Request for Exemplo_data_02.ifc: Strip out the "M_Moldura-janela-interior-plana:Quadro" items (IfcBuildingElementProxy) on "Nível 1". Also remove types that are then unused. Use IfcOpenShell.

First a look at what the model holds.

```python
import ifcopenshell
import ifcopenshell.util.element

model = ifcopenshell.open("Exemplo_data_02.ifc")
print(model.schema)
storey = next(s for s in model.by_type("IfcBuildingStorey") if s.Name == "Nível 1")
proxies = [e for e in ifcopenshell.util.element.get_decomposition(storey) if e.is_a("IfcBuildingElementProxy")]
seen = {}
for e in proxies:
    element_type = ifcopenshell.util.element.get_type(e)
    name = element_type.Name if element_type not in (None, e) else None
    seen[name] = seen.get(name, 0) + 1
for name, count in sorted(seen.items(), key=str):
    print(count, "x", name)
```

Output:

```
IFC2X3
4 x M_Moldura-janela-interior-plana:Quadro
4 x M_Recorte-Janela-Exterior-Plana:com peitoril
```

```python
import ifcopenshell
import ifcopenshell.api.root
import ifcopenshell.util.element

model = ifcopenshell.open("Exemplo_data_02.ifc")

storey = next(s for s in model.by_type("IfcBuildingStorey") if s.Name == "Nível 1")
proxies = [e for e in ifcopenshell.util.element.get_decomposition(storey) if e.is_a("IfcBuildingElementProxy")]
targets = [e for e in proxies if (t := ifcopenshell.util.element.get_type(e)) not in (None, e) and t.Name == "M_Moldura-janela-interior-plana:Quadro"]
types = {ifcopenshell.util.element.get_type(e) for e in targets} - {None, *targets}

for e in targets:
    ifcopenshell.api.root.remove_product(model, product=e)
print(len(targets), "removed")

unused = [t for t in types if not ifcopenshell.util.element.get_types(t)]
for t in unused:
    ifcopenshell.api.root.remove_product(model, product=t)
print(len(unused), "unused types removed")

model.write("Exemplo_data_02_edited.ifc")
```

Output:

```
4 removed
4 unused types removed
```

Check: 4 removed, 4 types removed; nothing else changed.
